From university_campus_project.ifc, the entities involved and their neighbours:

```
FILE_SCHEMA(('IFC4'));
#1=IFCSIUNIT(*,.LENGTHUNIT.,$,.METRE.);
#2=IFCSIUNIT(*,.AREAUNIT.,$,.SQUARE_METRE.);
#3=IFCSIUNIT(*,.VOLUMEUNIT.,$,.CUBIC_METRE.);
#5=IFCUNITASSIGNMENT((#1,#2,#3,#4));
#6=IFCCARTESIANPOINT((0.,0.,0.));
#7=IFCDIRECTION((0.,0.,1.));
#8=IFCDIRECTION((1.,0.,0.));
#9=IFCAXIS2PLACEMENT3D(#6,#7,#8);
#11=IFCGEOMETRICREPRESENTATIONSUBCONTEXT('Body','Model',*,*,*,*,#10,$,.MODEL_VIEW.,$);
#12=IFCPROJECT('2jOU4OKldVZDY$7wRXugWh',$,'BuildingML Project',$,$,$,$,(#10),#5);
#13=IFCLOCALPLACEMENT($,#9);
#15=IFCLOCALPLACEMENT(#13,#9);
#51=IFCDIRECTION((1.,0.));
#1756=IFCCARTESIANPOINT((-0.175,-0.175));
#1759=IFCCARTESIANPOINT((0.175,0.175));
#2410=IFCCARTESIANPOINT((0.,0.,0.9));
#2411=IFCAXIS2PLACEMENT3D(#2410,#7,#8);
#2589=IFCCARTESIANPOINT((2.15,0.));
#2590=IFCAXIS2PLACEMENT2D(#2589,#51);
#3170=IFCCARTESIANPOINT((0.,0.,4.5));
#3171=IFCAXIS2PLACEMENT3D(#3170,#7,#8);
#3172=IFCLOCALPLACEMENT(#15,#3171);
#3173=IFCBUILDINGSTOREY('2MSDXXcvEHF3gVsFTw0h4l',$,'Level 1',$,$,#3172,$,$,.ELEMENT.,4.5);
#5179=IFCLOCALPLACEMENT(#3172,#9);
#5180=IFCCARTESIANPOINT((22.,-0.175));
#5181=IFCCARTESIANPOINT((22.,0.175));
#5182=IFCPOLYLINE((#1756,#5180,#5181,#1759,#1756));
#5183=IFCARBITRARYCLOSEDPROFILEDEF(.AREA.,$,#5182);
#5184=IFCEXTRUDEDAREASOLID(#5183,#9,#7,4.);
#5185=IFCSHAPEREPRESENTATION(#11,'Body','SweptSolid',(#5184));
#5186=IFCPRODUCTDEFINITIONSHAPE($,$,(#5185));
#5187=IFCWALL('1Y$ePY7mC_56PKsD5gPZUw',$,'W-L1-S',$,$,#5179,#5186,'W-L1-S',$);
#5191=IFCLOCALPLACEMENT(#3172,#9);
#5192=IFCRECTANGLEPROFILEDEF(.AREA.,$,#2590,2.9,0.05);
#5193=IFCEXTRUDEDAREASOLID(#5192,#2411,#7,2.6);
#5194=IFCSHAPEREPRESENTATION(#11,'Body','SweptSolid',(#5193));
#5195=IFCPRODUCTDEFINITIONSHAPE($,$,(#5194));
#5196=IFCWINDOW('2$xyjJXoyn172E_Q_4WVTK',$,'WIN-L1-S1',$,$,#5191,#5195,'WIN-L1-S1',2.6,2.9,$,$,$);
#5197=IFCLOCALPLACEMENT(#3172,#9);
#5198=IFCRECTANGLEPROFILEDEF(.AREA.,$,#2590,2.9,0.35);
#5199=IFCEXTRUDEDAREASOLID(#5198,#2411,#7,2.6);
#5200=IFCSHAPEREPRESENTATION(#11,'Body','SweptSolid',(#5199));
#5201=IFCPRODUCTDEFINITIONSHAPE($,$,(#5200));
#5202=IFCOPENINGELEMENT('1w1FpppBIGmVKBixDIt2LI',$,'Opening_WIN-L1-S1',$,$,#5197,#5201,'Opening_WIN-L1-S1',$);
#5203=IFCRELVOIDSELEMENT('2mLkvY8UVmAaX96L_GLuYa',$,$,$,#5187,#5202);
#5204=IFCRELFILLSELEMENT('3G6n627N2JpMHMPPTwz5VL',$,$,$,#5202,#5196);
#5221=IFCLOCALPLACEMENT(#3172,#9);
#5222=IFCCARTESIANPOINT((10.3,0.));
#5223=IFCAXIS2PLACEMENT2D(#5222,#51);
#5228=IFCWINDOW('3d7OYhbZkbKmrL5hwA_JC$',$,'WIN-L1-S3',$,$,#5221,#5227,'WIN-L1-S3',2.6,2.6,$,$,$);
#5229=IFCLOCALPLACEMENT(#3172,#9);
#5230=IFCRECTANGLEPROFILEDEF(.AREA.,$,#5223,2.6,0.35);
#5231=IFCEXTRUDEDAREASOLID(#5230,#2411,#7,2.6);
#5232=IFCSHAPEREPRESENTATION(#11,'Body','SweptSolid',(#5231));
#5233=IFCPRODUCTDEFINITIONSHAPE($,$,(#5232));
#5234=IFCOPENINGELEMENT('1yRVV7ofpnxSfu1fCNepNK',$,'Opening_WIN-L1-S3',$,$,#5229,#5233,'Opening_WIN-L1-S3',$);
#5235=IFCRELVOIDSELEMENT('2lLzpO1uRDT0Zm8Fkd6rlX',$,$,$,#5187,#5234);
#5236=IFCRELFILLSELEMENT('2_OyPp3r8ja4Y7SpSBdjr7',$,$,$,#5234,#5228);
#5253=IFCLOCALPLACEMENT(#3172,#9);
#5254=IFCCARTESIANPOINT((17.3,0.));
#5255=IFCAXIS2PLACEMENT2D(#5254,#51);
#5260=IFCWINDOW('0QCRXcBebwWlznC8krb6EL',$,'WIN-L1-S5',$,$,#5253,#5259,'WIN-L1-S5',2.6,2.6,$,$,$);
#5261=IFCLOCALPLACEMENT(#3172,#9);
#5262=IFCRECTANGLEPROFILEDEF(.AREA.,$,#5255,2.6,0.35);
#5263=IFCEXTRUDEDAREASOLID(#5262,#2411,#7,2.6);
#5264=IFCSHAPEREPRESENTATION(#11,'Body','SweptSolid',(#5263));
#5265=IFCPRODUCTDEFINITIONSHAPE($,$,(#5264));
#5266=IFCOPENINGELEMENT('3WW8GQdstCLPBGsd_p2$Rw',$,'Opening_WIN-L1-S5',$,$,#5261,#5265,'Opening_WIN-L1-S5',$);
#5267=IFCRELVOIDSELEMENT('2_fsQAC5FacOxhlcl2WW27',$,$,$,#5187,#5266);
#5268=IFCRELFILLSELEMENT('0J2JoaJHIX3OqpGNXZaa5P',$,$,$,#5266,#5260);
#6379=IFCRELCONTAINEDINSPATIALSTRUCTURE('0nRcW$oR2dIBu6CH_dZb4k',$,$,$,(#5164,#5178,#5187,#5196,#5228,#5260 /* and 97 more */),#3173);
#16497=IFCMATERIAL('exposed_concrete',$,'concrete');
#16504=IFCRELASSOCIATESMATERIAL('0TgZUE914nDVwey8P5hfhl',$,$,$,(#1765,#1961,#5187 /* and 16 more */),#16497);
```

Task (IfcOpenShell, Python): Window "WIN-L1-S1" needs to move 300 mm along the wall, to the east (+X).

```python
import ifcopenshell
import ifcopenshell.api.geometry
import ifcopenshell.util.placement

model = ifcopenshell.open("university_campus_project.ifc")

window = model.by_guid("2$xyjJXoyn172E_Q_4WVTK")
opening = window.FillsVoids[0].RelatingOpeningElement
wall = opening.VoidsElements[0].RelatingBuildingElement

wall_matrix = ifcopenshell.util.placement.get_local_placement(wall.ObjectPlacement)
shift = wall_matrix[:3, 0] * 0.3
before = ifcopenshell.util.placement.get_local_placement(window.ObjectPlacement)[:3, 3].copy()

# The window is not placed relative to its opening, so move both.
for product in (opening, window):
    matrix = ifcopenshell.util.placement.get_local_placement(product.ObjectPlacement)
    matrix[:3, 3] += shift
    ifcopenshell.api.geometry.edit_object_placement(model, product=product, matrix=matrix, is_si=False)

after = ifcopenshell.util.placement.get_local_placement(window.ObjectPlacement)[:3, 3]
print("window moved by", (after - before).round(3) + 0.0)

model.write("university_campus_project-out.ifc")
```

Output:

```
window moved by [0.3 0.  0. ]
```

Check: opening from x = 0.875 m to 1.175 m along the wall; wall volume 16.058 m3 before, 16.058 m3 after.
